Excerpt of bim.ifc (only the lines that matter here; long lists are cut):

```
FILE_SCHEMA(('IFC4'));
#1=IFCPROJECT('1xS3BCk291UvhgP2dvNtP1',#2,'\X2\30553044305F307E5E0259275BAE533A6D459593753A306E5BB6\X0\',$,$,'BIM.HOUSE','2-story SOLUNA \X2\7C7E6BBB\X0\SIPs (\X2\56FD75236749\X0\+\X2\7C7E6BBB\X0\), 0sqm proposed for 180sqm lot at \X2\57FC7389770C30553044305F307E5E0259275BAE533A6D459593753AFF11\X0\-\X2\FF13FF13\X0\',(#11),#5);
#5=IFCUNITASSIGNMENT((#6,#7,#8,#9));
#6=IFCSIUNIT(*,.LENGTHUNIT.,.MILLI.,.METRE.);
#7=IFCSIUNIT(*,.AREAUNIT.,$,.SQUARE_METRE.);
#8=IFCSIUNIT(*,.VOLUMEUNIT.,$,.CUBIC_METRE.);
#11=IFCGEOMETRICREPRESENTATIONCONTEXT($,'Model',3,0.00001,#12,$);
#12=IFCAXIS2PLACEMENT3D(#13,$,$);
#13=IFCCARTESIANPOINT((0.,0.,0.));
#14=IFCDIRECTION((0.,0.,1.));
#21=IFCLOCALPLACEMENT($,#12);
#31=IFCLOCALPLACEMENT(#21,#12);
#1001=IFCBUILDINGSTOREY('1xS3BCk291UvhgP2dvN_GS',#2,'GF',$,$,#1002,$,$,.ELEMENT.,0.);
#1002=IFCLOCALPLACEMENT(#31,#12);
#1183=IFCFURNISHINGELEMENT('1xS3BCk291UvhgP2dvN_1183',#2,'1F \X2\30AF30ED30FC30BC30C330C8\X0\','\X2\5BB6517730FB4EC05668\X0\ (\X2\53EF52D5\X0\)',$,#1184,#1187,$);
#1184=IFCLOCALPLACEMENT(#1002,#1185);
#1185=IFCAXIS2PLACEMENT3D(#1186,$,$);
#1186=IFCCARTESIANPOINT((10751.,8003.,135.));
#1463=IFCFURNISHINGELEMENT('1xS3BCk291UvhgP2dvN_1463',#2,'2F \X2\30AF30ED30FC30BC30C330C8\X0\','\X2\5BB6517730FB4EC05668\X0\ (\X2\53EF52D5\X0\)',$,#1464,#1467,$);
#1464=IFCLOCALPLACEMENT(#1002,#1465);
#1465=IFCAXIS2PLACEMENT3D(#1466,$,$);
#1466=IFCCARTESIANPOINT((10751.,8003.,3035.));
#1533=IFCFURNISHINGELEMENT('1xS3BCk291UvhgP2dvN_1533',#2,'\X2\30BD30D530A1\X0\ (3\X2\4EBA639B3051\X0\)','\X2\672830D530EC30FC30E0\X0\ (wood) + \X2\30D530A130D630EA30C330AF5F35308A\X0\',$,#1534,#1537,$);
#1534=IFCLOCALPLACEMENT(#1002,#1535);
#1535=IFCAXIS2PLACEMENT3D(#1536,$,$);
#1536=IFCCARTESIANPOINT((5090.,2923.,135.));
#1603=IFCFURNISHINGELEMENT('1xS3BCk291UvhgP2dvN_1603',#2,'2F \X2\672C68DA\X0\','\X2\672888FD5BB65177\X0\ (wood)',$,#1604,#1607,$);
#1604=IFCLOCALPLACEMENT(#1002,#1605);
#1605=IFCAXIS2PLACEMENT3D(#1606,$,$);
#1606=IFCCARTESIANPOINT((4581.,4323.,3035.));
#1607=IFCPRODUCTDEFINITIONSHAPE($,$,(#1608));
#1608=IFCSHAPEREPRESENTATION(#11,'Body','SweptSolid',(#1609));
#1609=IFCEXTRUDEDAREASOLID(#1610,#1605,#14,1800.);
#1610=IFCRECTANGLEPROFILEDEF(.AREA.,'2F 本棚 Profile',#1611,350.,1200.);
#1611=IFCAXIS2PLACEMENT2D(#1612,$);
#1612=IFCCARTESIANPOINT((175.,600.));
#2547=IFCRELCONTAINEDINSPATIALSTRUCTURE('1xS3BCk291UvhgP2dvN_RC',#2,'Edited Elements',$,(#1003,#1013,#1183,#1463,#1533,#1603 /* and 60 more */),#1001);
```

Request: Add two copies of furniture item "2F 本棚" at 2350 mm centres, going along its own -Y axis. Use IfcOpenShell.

```python
import ifcopenshell
import ifcopenshell.api.geometry
import ifcopenshell.api.root
import ifcopenshell.util.element
import ifcopenshell.util.placement

model = ifcopenshell.open("bim.ifc")


def reuse_history(source, copy):
    """copy_class also copies each property set's owner history, people and application; keep the originals."""
    for rel in copy.IsDefinedBy:
        if rel.is_a("IfcRelDefinesByProperties") and (history := rel.RelatingPropertyDefinition.OwnerHistory):
            rel.RelatingPropertyDefinition.OwnerHistory = source.OwnerHistory
            ifcopenshell.util.element.remove_deep2(model, history)


source = model.by_guid("1xS3BCk291UvhgP2dvN_1603")
base = ifcopenshell.util.placement.get_local_placement(source.ObjectPlacement)
step = -base[:3, 1] * 2350.0

for i in range(1, 3):
    copy = ifcopenshell.api.root.copy_class(model, product=source)
    copy.Representation = ifcopenshell.util.element.copy_deep(
        model, source.Representation, exclude=["IfcGeometricRepresentationContext", "IfcRepresentationMap"]
    )
    reuse_history(source, copy)
    matrix = base.copy()
    matrix[:3, 3] += i * step
    print("added at", matrix[:3, 3].round(3) + 0.0)
    ifcopenshell.api.geometry.edit_object_placement(model, product=copy, matrix=matrix, is_si=False)

model.write("bim_rev.ifc")
```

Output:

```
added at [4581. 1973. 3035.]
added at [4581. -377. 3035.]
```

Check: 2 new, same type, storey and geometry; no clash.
